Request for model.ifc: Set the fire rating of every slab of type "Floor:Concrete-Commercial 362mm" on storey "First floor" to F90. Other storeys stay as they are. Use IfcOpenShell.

First a look at what the model holds.

```python
import ifcopenshell
import ifcopenshell.util.element

model = ifcopenshell.open("model.ifc")
print(model.schema)
storey = next(s for s in model.by_type("IfcBuildingStorey") if s.Name == "First floor")
slabs = [e for e in ifcopenshell.util.element.get_decomposition(storey) if e.is_a("IfcSlab")]
seen = {}
for e in slabs:
    element_type = ifcopenshell.util.element.get_type(e)
    key = (element_type.Name if element_type != e and element_type else None, ifcopenshell.util.element.get_pset(e, "Pset_SlabCommon", "FireRating"))
    seen[key] = seen.get(key, 0) + 1
for (name, value), count in sorted(seen.items(), key=str):
    print(count, "x", name, "|", value)
```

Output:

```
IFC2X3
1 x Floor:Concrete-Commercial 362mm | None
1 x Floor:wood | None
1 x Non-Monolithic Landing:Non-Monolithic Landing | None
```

```python
import ifcopenshell
import ifcopenshell.api.pset
import ifcopenshell.util.element

model = ifcopenshell.open("model.ifc")

storey = next(s for s in model.by_type("IfcBuildingStorey") if s.Name == "First floor")
slabs = [e for e in ifcopenshell.util.element.get_decomposition(storey) if e.is_a("IfcSlab")]

count = 0
for e in slabs:
    element_type = ifcopenshell.util.element.get_type(e)
    if element_type in (None, e) or element_type.Name != "Floor:Concrete-Commercial 362mm":
        continue
    # add_pset returns the element's existing set when there is one.
    pset = ifcopenshell.api.pset.add_pset(model, product=e, name="Pset_SlabCommon")
    ifcopenshell.api.pset.edit_pset(model, pset=pset, properties={"FireRating": "F90"})
    count += 1

print(count, "slabs updated")

model.write("model_edited.ifc")
```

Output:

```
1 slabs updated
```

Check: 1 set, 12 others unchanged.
